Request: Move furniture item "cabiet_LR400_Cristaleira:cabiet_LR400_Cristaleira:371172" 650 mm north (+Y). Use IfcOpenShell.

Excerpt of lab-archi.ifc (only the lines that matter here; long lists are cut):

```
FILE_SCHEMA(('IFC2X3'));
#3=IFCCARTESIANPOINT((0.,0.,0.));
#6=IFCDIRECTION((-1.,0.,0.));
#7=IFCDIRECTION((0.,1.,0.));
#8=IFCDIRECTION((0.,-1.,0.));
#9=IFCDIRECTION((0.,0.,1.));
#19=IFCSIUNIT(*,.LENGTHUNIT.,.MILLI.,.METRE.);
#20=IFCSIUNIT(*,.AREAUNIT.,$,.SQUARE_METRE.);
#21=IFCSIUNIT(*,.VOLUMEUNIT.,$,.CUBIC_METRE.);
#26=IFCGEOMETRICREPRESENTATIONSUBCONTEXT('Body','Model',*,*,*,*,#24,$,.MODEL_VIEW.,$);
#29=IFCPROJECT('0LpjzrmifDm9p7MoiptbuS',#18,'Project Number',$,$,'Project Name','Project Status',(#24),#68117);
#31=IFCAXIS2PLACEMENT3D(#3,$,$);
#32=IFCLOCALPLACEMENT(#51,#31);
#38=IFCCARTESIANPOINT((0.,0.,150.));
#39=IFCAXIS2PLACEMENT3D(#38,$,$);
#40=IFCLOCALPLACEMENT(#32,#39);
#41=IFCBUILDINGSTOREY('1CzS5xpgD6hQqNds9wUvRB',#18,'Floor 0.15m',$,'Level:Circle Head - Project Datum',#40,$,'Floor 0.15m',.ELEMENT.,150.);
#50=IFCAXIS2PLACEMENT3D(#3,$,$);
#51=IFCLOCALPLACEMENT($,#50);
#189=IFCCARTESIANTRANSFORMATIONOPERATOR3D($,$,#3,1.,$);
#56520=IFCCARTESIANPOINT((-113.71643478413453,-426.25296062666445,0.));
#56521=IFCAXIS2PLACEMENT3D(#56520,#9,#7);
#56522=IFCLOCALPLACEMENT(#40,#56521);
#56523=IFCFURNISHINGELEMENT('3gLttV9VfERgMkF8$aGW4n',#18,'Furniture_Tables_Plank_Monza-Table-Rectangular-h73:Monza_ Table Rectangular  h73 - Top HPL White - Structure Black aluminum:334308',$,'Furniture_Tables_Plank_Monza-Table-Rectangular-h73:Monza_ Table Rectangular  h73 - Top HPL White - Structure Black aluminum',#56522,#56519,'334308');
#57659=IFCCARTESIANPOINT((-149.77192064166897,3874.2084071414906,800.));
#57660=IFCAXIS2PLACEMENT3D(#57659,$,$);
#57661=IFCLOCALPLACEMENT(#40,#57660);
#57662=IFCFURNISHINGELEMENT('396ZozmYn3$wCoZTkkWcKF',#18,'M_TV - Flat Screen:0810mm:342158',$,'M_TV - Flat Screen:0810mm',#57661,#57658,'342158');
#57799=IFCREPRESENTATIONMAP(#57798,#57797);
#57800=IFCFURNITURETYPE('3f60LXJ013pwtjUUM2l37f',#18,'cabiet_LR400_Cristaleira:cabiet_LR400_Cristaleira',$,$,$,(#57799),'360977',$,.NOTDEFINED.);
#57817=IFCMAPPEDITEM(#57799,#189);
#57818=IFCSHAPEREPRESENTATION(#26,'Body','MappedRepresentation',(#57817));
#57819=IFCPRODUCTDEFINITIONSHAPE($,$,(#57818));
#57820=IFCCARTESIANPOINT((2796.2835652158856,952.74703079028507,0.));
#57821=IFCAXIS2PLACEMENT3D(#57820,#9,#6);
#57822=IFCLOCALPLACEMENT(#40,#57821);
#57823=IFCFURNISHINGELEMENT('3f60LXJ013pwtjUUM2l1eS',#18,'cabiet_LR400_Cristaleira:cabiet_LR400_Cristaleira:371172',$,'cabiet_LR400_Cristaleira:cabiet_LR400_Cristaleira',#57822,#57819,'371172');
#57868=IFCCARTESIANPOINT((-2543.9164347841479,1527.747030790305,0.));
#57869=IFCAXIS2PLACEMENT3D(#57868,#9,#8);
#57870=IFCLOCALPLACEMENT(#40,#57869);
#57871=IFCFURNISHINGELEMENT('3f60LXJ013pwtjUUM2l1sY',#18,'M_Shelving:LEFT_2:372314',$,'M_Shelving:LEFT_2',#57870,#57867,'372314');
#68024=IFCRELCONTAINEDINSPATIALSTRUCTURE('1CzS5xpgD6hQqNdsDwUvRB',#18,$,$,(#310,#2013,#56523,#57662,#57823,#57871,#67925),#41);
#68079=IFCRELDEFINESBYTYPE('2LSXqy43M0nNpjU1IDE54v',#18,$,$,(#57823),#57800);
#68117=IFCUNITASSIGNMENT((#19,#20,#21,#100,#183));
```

```python
import ifcopenshell
import ifcopenshell.api.geometry
import ifcopenshell.util.placement

model = ifcopenshell.open("lab-archi.ifc")

item = model.by_guid("3f60LXJ013pwtjUUM2l1eS")
matrix = ifcopenshell.util.placement.get_local_placement(item.ObjectPlacement)
matrix[1, 3] += 650.0
ifcopenshell.api.geometry.edit_object_placement(model, product=item, matrix=matrix, is_si=False)

print(ifcopenshell.util.placement.get_local_placement(item.ObjectPlacement).round(3) + 0.0)

model.write("lab-archi_updated.ifc")
```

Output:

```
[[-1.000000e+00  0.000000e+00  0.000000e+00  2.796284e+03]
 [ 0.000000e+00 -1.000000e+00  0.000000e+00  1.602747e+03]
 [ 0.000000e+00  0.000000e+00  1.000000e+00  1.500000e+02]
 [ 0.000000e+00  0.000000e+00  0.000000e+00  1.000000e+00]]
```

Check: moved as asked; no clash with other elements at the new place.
